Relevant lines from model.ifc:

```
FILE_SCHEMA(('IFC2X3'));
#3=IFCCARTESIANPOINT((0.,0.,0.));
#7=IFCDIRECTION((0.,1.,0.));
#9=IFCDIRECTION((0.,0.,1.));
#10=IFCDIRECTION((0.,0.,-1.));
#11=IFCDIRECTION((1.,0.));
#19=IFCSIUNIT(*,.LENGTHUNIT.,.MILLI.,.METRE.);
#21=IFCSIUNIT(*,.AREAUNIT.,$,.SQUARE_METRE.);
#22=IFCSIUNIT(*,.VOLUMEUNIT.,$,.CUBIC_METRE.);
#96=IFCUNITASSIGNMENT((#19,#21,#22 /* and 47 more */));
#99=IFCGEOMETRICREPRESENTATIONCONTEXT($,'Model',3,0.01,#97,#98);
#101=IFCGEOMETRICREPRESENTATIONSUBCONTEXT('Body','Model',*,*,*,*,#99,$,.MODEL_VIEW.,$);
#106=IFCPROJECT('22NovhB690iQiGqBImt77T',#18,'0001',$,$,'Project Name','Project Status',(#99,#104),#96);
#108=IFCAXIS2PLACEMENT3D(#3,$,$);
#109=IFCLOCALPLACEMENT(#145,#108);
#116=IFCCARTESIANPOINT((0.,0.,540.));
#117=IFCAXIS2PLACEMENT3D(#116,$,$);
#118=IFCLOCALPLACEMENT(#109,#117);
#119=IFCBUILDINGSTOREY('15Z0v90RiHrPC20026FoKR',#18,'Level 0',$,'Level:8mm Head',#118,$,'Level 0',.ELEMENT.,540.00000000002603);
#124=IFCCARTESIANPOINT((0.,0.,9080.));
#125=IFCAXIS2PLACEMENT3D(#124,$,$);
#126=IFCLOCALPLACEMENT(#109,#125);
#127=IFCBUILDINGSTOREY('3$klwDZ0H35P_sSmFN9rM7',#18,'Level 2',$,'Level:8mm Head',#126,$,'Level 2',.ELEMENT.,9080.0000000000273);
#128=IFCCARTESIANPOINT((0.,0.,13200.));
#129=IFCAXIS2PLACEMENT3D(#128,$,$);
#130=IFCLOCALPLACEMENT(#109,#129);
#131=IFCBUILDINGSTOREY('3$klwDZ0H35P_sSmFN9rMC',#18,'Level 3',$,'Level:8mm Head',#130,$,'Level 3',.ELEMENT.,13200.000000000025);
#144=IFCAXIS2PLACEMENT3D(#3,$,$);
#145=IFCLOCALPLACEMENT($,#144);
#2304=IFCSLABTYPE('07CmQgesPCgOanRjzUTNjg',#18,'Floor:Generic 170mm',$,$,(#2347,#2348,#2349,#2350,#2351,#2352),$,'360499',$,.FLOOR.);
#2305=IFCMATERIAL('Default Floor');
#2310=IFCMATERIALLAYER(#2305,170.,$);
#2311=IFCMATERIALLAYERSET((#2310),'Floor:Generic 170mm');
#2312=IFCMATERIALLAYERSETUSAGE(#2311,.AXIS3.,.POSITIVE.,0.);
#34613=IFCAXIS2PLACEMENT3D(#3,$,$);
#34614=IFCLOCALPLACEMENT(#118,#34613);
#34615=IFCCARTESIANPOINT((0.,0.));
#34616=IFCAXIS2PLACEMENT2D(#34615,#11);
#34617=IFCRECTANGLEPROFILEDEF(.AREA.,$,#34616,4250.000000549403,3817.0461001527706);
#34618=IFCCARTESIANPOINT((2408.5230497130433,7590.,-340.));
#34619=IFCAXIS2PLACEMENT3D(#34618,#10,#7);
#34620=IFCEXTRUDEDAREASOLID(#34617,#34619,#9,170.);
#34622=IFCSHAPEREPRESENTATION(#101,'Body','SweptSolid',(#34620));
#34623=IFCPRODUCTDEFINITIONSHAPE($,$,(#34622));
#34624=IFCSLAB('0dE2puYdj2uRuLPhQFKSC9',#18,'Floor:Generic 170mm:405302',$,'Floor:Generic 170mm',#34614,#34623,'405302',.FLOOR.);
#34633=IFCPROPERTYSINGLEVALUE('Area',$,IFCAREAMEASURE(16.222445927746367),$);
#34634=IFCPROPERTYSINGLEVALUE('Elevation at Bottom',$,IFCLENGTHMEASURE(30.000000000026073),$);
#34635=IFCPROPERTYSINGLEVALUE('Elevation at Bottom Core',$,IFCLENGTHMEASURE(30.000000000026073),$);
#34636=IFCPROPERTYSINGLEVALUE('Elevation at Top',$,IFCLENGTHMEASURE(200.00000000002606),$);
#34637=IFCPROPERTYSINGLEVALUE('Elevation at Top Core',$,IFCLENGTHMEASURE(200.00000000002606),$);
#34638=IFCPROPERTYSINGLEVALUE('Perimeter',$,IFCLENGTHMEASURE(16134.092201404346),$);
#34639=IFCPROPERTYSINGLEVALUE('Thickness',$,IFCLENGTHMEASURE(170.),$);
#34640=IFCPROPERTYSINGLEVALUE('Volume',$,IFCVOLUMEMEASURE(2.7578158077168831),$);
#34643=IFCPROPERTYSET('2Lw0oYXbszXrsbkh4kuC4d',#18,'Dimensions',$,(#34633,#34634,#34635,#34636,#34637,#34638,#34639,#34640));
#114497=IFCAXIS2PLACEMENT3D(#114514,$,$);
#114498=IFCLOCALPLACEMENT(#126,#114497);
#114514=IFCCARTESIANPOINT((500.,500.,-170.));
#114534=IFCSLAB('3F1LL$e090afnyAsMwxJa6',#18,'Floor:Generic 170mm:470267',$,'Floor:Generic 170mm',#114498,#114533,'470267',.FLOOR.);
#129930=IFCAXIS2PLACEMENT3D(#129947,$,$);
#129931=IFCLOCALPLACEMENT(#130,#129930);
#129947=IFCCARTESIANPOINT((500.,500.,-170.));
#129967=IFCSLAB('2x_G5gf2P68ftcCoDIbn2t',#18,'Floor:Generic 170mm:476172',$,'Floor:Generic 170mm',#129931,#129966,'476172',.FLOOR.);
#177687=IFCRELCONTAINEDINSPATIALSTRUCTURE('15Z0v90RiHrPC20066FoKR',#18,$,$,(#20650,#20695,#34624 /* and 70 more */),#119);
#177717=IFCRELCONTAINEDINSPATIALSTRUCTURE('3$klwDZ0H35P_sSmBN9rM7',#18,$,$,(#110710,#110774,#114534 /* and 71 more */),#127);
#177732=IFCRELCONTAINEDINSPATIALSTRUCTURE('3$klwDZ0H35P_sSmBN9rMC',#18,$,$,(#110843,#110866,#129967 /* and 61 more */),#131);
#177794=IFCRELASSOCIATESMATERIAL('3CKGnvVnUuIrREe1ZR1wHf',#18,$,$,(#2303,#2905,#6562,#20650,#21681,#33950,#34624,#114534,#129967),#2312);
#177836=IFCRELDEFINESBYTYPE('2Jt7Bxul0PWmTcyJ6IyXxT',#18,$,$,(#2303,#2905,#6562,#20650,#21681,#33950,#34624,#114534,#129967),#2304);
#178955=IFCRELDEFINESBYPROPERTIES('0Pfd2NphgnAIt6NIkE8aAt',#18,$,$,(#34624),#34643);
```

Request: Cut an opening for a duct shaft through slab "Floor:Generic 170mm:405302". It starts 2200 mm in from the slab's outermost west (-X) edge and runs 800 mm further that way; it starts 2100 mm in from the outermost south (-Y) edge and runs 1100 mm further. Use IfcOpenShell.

```python
import numpy as np
import ifcopenshell
import ifcopenshell.api.feature
import ifcopenshell.api.geometry
import ifcopenshell.api.pset
import ifcopenshell.api.root
import ifcopenshell.geom
import ifcopenshell.util.element
import ifcopenshell.util.placement
import ifcopenshell.util.representation
import ifcopenshell.util.shape
import ifcopenshell.util.unit

model = ifcopenshell.open("model.ifc")
unit_scale = ifcopenshell.util.unit.calculate_unit_scale(model)
area_scale = ifcopenshell.util.unit.calculate_unit_scale(model, "AREAUNIT")
volume_scale = ifcopenshell.util.unit.calculate_unit_scale(model, "VOLUMEUNIT")
settings = ifcopenshell.geom.settings()


def volume(element):
    """Net volume in cubic metres, openings subtracted."""
    shape = ifcopenshell.geom.create_shape(settings, element)
    return ifcopenshell.util.shape.get_volume(shape.geometry)


slab = model.by_id(34624)
before = volume(slab)

# Extent in the slab's own axes, in metres. The edges named are its -X and -Y sides.
slab_shape = ifcopenshell.geom.create_shape(settings, slab)
vertices = ifcopenshell.util.shape.get_vertices(slab_shape.geometry)
x_min, y_min, bottom = vertices.min(axis=0)
top = vertices[:, 2].max()

opening = ifcopenshell.api.root.create_entity(model, ifc_class="IfcOpeningElement", name="Duct shaft opening")
context = ifcopenshell.util.representation.get_context(model, "Model", "Body", "MODEL_VIEW")
width, depth = 0.8, 1.1
outline = [(0.0, 0.0), (width, 0.0), (width, depth), (0.0, depth), (0.0, 0.0)]
# Overshoot both faces by 50 mm so the cut is clean.
shape = ifcopenshell.api.geometry.add_slab_representation(
    model, context=context, depth=top - bottom + 0.1, polyline=outline
)
ifcopenshell.api.geometry.assign_representation(model, product=opening, representation=shape)

matrix = ifcopenshell.util.placement.get_local_placement(slab.ObjectPlacement)
matrix[:, 3] = matrix @ np.append(np.array([x_min + 2.2, y_min + 2.1, bottom - 0.05]) / unit_scale, 1.0)
ifcopenshell.api.geometry.edit_object_placement(model, product=opening, matrix=matrix, is_si=False)
ifcopenshell.api.feature.add_feature(model, feature=opening, element=slab)

after = volume(slab)

# Update the slab's stored quantities.
pset = model.by_id(ifcopenshell.util.element.get_pset(slab, "Dimensions", should_inherit=False)["id"])
ifcopenshell.api.pset.edit_pset(model, pset=pset, properties={
    "Area": model.create_entity("IfcAreaMeasure", after / (top - bottom) / area_scale),
    "Volume": model.create_entity("IfcVolumeMeasure", after / volume_scale),
})

print(f"slab volume {before:.3f} -> {after:.3f} m3")

model.write("model_updated.ifc")
```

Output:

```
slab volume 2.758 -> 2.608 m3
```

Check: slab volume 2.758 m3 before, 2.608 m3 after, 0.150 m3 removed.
